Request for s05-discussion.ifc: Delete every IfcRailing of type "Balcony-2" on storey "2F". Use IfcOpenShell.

First a look at what the model holds.

```python
import ifcopenshell
import ifcopenshell.util.element

model = ifcopenshell.open("s05-discussion.ifc")
print(model.schema)
storey = next(s for s in model.by_type("IfcBuildingStorey") if s.Name == "2F")
railings = [e for e in ifcopenshell.util.element.get_decomposition(storey) if e.is_a("IfcRailing")]
seen = {}
for e in railings:
    element_type = ifcopenshell.util.element.get_type(e)
    name = element_type.Name if element_type not in (None, e) else None
    seen[name] = seen.get(name, 0) + 1
for name, count in sorted(seen.items(), key=str):
    print(count, "x", name)
```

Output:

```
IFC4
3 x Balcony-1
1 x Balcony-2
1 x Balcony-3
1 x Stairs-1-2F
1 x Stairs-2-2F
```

```python
import ifcopenshell
import ifcopenshell.api.root
import ifcopenshell.util.element

model = ifcopenshell.open("s05-discussion.ifc")

storey = next(s for s in model.by_type("IfcBuildingStorey") if s.Name == "2F")
railings = [e for e in ifcopenshell.util.element.get_decomposition(storey) if e.is_a("IfcRailing")]
targets = [e for e in railings if (t := ifcopenshell.util.element.get_type(e)) not in (None, e) and t.Name == "Balcony-2"]

for e in targets:
    ifcopenshell.api.root.remove_product(model, product=e)
print(len(targets), "removed")

model.write("s05-discussion_v2.ifc")
```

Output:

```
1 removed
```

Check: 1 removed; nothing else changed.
